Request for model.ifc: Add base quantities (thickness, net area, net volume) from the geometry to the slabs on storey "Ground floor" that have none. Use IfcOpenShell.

First a look at what the model holds.

```python
import ifcopenshell
import ifcopenshell.util.element
import ifcopenshell.util.unit

model = ifcopenshell.open("model.ifc")
print(model.schema)
for unit_type in ("LENGTHUNIT", "AREAUNIT", "VOLUMEUNIT"):
    print(unit_type, ifcopenshell.util.unit.calculate_unit_scale(model, unit_type))
storey = next(s for s in model.by_type("IfcBuildingStorey") if s.Name == "Ground floor")
slabs = [e for e in ifcopenshell.util.element.get_decomposition(storey) if e.is_a("IfcSlab")]
for e in sorted(slabs, key=lambda e: e.id()):
    print(e.id(), e.is_a(), e.Name, list(ifcopenshell.util.element.get_psets(e, qtos_only=True)), sep=" | ")
```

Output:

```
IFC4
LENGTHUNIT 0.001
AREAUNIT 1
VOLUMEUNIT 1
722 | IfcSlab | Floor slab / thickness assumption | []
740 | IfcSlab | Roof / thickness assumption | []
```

```python
import ifcopenshell
import ifcopenshell.api.pset
import ifcopenshell.geom
import ifcopenshell.util.element
import ifcopenshell.util.shape
import ifcopenshell.util.unit

model = ifcopenshell.open("model.ifc")
unit_scale = ifcopenshell.util.unit.calculate_unit_scale(model)
area_scale = ifcopenshell.util.unit.calculate_unit_scale(model, "AREAUNIT")
volume_scale = ifcopenshell.util.unit.calculate_unit_scale(model, "VOLUMEUNIT")
settings = ifcopenshell.geom.settings()

storey = next(s for s in model.by_type("IfcBuildingStorey") if s.Name == "Ground floor")
slabs = [e for e in ifcopenshell.util.element.get_decomposition(storey) if e.is_a("IfcSlab")]

for e in sorted(slabs, key=lambda e: e.id()):
    if ifcopenshell.util.element.get_psets(e, qtos_only=True, should_inherit=False):
        continue
    # Geometry comes back in metres, in the element's own axes.
    shape = ifcopenshell.geom.create_shape(settings, e)
    values = {
        "Width": ifcopenshell.util.shape.get_z(shape.geometry) / unit_scale,
        "NetArea": ifcopenshell.util.shape.get_footprint_area(shape.geometry) / area_scale,
        "NetVolume": ifcopenshell.util.shape.get_volume(shape.geometry) / volume_scale,
    }
    qto = ifcopenshell.api.pset.add_qto(model, product=e, name="Qto_SlabBaseQuantities")
    ifcopenshell.api.pset.edit_qto(model, qto=qto, properties=values)
    print(e.id(), {k: round(v, 3) for k, v in values.items()})

model.write("model-out.ifc")
```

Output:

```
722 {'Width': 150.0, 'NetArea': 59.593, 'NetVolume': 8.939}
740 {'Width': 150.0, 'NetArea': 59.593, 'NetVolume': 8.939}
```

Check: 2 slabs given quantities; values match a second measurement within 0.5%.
